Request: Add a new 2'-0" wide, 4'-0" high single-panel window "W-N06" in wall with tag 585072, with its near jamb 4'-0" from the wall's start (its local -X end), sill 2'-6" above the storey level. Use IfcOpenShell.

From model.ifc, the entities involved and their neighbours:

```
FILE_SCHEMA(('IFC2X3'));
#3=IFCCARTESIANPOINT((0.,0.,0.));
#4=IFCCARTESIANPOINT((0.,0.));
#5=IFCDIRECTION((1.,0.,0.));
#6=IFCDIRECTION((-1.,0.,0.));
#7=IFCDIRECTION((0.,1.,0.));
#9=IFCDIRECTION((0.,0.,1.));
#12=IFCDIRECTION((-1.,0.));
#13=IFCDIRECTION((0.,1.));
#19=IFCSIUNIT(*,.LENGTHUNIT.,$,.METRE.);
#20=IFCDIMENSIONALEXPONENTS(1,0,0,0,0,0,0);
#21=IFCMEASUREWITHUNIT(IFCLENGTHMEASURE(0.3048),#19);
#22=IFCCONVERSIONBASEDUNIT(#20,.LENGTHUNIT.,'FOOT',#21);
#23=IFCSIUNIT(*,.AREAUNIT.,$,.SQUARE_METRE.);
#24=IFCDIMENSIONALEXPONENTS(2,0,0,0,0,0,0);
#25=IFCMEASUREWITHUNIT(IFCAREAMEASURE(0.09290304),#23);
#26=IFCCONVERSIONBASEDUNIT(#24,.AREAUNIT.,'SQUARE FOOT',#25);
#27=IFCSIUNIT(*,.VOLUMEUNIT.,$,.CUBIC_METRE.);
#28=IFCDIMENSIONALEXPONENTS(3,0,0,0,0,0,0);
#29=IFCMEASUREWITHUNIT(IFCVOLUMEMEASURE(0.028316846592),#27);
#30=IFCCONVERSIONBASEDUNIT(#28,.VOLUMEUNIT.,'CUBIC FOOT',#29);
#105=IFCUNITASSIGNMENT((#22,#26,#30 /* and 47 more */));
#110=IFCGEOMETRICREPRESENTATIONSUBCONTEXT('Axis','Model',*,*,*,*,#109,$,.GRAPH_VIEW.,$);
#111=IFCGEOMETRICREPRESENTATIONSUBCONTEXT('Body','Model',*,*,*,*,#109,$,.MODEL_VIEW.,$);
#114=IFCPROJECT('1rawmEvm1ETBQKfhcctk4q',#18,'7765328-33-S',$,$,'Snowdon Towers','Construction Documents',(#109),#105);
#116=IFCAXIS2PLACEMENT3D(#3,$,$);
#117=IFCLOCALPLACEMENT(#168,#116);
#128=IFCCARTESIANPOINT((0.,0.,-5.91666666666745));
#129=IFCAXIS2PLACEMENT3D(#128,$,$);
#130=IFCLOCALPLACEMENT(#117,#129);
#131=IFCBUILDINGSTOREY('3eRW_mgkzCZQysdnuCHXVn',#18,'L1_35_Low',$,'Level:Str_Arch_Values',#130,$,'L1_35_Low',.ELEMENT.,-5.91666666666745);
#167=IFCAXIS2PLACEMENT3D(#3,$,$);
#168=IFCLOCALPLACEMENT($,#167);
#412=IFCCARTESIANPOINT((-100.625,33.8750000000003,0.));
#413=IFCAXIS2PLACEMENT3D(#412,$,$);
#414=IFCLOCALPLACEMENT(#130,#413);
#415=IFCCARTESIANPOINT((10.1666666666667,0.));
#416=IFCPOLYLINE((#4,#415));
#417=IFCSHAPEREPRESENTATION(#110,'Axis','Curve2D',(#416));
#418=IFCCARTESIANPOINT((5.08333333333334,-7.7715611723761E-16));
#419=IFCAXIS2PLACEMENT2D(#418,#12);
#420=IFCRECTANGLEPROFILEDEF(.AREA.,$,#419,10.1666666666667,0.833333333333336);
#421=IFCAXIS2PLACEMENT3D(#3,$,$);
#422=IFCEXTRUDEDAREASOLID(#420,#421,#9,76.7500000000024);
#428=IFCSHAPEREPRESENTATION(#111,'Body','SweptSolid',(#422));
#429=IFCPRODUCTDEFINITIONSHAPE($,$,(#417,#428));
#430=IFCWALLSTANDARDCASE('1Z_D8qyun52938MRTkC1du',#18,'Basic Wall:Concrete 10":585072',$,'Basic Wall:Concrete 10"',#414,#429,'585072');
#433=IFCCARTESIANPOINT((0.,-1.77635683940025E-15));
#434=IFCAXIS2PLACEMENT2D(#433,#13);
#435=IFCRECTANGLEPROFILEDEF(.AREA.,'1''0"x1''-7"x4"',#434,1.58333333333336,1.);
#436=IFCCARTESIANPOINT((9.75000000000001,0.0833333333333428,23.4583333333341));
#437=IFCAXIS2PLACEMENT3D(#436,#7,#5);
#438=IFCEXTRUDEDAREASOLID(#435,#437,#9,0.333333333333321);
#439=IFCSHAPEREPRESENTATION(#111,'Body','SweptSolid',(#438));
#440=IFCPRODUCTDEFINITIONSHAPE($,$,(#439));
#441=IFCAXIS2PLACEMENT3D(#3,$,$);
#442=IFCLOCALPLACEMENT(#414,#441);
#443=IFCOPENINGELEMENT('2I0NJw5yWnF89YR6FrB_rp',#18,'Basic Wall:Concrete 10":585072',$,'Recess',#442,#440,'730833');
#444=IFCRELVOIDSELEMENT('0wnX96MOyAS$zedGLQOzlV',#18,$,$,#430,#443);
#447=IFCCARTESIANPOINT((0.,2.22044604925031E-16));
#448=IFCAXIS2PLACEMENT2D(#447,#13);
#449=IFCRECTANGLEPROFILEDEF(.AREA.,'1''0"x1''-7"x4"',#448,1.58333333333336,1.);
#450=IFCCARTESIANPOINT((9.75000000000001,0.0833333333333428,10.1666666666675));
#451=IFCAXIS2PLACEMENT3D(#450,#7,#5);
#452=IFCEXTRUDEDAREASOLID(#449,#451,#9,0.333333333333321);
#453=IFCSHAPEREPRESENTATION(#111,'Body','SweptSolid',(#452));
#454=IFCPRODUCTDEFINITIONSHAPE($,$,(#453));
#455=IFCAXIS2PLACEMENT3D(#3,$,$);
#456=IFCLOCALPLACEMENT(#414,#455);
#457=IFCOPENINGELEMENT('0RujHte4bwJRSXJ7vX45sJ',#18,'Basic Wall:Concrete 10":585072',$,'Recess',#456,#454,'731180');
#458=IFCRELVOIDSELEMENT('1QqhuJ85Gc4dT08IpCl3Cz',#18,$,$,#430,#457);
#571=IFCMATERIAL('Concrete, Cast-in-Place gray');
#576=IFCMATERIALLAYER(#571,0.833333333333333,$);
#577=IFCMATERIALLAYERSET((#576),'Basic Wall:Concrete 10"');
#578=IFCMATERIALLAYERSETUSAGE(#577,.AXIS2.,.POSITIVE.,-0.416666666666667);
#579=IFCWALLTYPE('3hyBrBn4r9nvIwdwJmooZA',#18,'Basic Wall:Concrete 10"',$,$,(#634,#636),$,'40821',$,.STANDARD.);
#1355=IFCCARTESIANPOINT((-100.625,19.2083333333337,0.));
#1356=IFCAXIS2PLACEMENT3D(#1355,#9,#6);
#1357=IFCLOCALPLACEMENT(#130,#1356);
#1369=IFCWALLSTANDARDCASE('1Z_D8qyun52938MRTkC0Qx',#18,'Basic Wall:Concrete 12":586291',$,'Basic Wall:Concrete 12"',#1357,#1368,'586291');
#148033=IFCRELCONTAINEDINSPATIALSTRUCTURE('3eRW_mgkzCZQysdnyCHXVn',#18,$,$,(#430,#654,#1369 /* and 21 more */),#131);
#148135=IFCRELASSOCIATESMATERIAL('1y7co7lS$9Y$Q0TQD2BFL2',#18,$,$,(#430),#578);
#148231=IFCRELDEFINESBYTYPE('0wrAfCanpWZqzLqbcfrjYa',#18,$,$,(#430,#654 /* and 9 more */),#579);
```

```python
import numpy as np
import ifcopenshell
import ifcopenshell.api.feature
import ifcopenshell.api.geometry
import ifcopenshell.api.root
import ifcopenshell.api.spatial
import ifcopenshell.api.type
import ifcopenshell.geom
import ifcopenshell.util.element
import ifcopenshell.util.placement
import ifcopenshell.util.representation
import ifcopenshell.util.shape
import ifcopenshell.util.unit

model = ifcopenshell.open("model.ifc")
unit_scale = ifcopenshell.util.unit.calculate_unit_scale(model)
settings = ifcopenshell.geom.settings()


def volume(element):
    """Net volume in cubic metres, openings subtracted."""
    shape = ifcopenshell.geom.create_shape(settings, element)
    return ifcopenshell.util.shape.get_volume(shape.geometry)


wall = model.by_guid("1Z_D8qyun52938MRTkC1du")
storey = ifcopenshell.util.element.get_container(wall, ifc_class="IfcBuildingStorey")
context = ifcopenshell.util.representation.get_context(model, "Model", "Body", "MODEL_VIEW")
before = volume(wall)

width, height, from_end, sill = 0.6096, 1.2192, 1.2192, 0.762  # metres

# The wall runs along its own X axis, and the end named is its -X end.
wall_shape = ifcopenshell.geom.create_shape(settings, wall)
x, y, z = ifcopenshell.util.shape.get_vertices(wall_shape.geometry).T
start = x.min() + from_end
face, thickness = float(y.min()), float(y.max() - y.min())
wall_matrix = ifcopenshell.util.placement.get_local_placement(wall.ObjectPlacement)
level = ifcopenshell.util.placement.get_local_placement(storey.ObjectPlacement)[2, 3]


def in_wall(x, y):
    """Placement at x, y metres in the wall's axes, at sill height."""
    matrix = wall_matrix.copy()
    matrix[:, 3] = wall_matrix @ np.array([x / unit_scale, y / unit_scale, 0.0, 1.0])
    matrix[2, 3] = level + sill / unit_scale
    return matrix


# Opening: a box that overshoots both wall faces by 50 mm.
opening = ifcopenshell.api.root.create_entity(model, ifc_class="IfcOpeningElement")
box = ifcopenshell.api.geometry.add_wall_representation(
    model, context=context, length=width, height=height, thickness=thickness + 0.1
)
ifcopenshell.api.geometry.assign_representation(model, product=opening, representation=box)
ifcopenshell.api.geometry.edit_object_placement(model, product=opening, matrix=in_wall(start, face - 0.05), is_si=False)
ifcopenshell.api.feature.add_feature(model, feature=opening, element=wall)

window = ifcopenshell.api.root.create_entity(model, ifc_class="IfcWindow", name="W-N06")
window.OverallWidth, window.OverallHeight = width / unit_scale, height / unit_scale
body = ifcopenshell.api.geometry.add_window_representation(
    model,
    context=context,
    overall_width=window.OverallWidth,
    overall_height=window.OverallHeight,
    partition_type="SINGLE_PANEL",
)
ifcopenshell.api.geometry.assign_representation(model, product=window, representation=body)
ifcopenshell.api.spatial.assign_container(model, products=[window], relating_structure=storey)
fills = ifcopenshell.api.feature.add_filling(model, opening=opening, element=window)
fills.OwnerHistory = window.OwnerHistory  # required in IFC2X3

# IFC2X3 keeps the operation on the window style.
style = ifcopenshell.api.root.create_entity(model, ifc_class="IfcWindowStyle", name="W-N06")
style.OperationType, style.ConstructionType = "SINGLE_PANEL", "NOTDEFINED"
style.ParameterTakesPrecedence = style.Sizeable = False
ifcopenshell.api.type.assign_type(model, related_objects=[window], relating_type=style)

# Centre the window in the wall's thickness.
ifcopenshell.api.geometry.edit_object_placement(model, product=window, matrix=in_wall(start, face), is_si=False)
window_shape = ifcopenshell.geom.create_shape(settings, window)
depth = ifcopenshell.util.shape.get_vertices(window_shape.geometry)[:, 1]
offset = face + thickness / 2 - (depth.min() + depth.max()) / 2
ifcopenshell.api.geometry.edit_object_placement(model, product=window, matrix=in_wall(start, offset), is_si=False)

after = volume(wall)

print(f"wall volume {before:.3f} -> {after:.3f} m3")

model.write("model_edited.ifc")
```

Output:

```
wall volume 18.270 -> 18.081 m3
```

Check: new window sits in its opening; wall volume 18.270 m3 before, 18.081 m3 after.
